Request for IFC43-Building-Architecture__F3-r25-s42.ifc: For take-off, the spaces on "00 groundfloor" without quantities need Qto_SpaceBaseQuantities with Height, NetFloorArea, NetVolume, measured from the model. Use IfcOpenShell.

First a look at what the model holds.

```python
import ifcopenshell
import ifcopenshell.util.element
import ifcopenshell.util.unit

model = ifcopenshell.open("IFC43-Building-Architecture__F3-r25-s42.ifc")
print(model.schema)
for unit_type in ("LENGTHUNIT", "AREAUNIT", "VOLUMEUNIT"):
    print(unit_type, ifcopenshell.util.unit.calculate_unit_scale(model, unit_type))
storey = next(s for s in model.by_type("IfcBuildingStorey") if s.Name == "00 groundfloor")
spaces = [e for e in ifcopenshell.util.element.get_decomposition(storey) if e.is_a("IfcSpace")]
for e in sorted(spaces, key=lambda e: e.id()):
    print(e.id(), e.is_a(), e.Name, list(ifcopenshell.util.element.get_psets(e, qtos_only=True)), sep=" | ")
```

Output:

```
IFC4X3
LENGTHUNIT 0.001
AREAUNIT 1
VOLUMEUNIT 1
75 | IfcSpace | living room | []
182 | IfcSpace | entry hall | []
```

```python
import ifcopenshell
import ifcopenshell.api.pset
import ifcopenshell.geom
import ifcopenshell.util.element
import ifcopenshell.util.shape
import ifcopenshell.util.unit

model = ifcopenshell.open("IFC43-Building-Architecture__F3-r25-s42.ifc")
unit_scale = ifcopenshell.util.unit.calculate_unit_scale(model)
area_scale = ifcopenshell.util.unit.calculate_unit_scale(model, "AREAUNIT")
volume_scale = ifcopenshell.util.unit.calculate_unit_scale(model, "VOLUMEUNIT")
settings = ifcopenshell.geom.settings()

storey = next(s for s in model.by_type("IfcBuildingStorey") if s.Name == "00 groundfloor")
spaces = [e for e in ifcopenshell.util.element.get_decomposition(storey) if e.is_a("IfcSpace")]

for e in sorted(spaces, key=lambda e: e.id()):
    if ifcopenshell.util.element.get_psets(e, qtos_only=True, should_inherit=False):
        continue
    # Geometry comes back in metres, in the element's own axes.
    shape = ifcopenshell.geom.create_shape(settings, e)
    values = {
        "Height": ifcopenshell.util.shape.get_z(shape.geometry) / unit_scale,
        "NetFloorArea": ifcopenshell.util.shape.get_footprint_area(shape.geometry) / area_scale,
        "NetVolume": ifcopenshell.util.shape.get_volume(shape.geometry) / volume_scale,
    }
    qto = ifcopenshell.api.pset.add_qto(model, product=e, name="Qto_SpaceBaseQuantities")
    ifcopenshell.api.pset.edit_qto(model, qto=qto, properties=values)
    print(e.id(), {k: round(v, 3) for k, v in values.items()})

model.write("IFC43-Building-Architecture__F3-r25-s42_updated.ifc")
```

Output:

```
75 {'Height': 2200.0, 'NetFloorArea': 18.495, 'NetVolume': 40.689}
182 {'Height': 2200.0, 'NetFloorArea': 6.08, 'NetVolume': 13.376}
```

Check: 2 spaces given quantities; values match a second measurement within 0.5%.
